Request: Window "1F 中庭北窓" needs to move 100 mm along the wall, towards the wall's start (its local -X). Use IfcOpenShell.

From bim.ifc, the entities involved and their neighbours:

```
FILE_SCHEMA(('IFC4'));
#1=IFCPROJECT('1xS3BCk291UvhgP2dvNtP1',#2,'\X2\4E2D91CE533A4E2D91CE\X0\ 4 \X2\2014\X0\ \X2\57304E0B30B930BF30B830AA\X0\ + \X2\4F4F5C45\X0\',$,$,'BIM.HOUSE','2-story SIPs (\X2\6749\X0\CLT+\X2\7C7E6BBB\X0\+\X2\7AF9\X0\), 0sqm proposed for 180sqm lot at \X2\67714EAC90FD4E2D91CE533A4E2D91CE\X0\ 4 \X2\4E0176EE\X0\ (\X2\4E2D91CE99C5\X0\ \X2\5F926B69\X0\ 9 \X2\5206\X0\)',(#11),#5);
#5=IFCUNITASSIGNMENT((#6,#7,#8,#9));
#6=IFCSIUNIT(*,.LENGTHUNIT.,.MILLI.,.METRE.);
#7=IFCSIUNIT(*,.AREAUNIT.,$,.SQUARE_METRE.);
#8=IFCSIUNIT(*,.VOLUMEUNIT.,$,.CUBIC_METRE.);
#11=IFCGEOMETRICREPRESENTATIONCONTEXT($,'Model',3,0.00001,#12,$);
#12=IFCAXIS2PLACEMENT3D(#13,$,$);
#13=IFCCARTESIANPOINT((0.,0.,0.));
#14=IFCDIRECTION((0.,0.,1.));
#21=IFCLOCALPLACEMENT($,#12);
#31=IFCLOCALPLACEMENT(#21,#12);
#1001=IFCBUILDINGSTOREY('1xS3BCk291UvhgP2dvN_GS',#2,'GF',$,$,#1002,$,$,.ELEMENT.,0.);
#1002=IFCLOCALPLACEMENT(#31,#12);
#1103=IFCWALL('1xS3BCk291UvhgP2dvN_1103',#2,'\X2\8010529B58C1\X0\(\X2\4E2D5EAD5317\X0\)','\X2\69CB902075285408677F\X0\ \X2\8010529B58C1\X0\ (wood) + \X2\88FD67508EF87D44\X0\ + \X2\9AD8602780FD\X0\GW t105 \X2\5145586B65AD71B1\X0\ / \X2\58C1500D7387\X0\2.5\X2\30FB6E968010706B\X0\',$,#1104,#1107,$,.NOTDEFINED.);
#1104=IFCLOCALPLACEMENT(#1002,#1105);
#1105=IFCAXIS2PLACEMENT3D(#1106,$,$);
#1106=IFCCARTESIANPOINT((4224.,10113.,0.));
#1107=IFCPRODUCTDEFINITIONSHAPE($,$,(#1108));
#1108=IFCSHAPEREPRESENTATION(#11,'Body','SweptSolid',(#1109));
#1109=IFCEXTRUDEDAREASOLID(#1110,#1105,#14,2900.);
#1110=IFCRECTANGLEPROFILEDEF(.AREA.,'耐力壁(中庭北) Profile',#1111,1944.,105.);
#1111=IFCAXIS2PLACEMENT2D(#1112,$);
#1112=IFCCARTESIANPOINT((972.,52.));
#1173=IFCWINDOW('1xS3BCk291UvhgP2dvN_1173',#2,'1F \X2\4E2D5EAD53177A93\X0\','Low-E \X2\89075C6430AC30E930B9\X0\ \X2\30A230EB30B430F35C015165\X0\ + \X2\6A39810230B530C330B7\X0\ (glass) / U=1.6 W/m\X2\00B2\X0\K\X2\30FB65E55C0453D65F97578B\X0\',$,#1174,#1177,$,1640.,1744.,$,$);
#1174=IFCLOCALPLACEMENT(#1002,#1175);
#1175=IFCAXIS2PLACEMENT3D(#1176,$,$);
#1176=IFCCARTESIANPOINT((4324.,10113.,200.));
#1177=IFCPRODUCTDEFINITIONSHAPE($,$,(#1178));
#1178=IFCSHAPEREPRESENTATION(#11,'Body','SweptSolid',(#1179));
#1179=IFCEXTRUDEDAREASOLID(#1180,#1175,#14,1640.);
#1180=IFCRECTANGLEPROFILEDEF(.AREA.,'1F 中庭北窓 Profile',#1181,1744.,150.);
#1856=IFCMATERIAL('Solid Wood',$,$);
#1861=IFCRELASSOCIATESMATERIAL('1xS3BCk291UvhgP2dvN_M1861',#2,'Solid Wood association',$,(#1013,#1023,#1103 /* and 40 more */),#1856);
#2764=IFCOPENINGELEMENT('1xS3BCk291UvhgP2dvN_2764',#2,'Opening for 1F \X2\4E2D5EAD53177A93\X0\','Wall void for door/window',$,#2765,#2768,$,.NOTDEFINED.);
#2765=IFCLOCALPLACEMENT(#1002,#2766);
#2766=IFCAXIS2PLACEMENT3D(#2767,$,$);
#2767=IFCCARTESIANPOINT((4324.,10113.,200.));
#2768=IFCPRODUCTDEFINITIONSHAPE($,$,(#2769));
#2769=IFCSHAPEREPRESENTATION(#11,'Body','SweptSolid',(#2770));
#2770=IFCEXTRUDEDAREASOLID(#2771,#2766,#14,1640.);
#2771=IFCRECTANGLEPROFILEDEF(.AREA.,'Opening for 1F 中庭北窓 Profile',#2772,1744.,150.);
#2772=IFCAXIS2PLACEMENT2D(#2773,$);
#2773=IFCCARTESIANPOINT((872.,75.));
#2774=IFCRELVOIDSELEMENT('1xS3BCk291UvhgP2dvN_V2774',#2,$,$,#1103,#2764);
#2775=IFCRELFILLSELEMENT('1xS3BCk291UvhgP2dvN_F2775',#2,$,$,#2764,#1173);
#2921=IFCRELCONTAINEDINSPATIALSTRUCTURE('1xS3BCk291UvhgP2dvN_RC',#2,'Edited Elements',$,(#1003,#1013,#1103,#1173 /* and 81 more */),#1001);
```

```python
import ifcopenshell
import ifcopenshell.api.geometry
import ifcopenshell.util.placement

model = ifcopenshell.open("bim.ifc")

window = model.by_guid("1xS3BCk291UvhgP2dvN_1173")
opening = window.FillsVoids[0].RelatingOpeningElement
wall = opening.VoidsElements[0].RelatingBuildingElement

wall_matrix = ifcopenshell.util.placement.get_local_placement(wall.ObjectPlacement)
shift = wall_matrix[:3, 0] * -100.0
before = ifcopenshell.util.placement.get_local_placement(window.ObjectPlacement)[:3, 3].copy()

# The window is not placed relative to its opening, so move both.
for product in (opening, window):
    matrix = ifcopenshell.util.placement.get_local_placement(product.ObjectPlacement)
    matrix[:3, 3] += shift
    ifcopenshell.api.geometry.edit_object_placement(model, product=product, matrix=matrix, is_si=False)

after = ifcopenshell.util.placement.get_local_placement(window.ObjectPlacement)[:3, 3]
print("window moved by", (after - before).round(3) + 0.0)

model.write("bim-out.ifc")
```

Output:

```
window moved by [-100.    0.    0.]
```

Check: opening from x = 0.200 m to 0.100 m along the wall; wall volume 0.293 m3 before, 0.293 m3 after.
